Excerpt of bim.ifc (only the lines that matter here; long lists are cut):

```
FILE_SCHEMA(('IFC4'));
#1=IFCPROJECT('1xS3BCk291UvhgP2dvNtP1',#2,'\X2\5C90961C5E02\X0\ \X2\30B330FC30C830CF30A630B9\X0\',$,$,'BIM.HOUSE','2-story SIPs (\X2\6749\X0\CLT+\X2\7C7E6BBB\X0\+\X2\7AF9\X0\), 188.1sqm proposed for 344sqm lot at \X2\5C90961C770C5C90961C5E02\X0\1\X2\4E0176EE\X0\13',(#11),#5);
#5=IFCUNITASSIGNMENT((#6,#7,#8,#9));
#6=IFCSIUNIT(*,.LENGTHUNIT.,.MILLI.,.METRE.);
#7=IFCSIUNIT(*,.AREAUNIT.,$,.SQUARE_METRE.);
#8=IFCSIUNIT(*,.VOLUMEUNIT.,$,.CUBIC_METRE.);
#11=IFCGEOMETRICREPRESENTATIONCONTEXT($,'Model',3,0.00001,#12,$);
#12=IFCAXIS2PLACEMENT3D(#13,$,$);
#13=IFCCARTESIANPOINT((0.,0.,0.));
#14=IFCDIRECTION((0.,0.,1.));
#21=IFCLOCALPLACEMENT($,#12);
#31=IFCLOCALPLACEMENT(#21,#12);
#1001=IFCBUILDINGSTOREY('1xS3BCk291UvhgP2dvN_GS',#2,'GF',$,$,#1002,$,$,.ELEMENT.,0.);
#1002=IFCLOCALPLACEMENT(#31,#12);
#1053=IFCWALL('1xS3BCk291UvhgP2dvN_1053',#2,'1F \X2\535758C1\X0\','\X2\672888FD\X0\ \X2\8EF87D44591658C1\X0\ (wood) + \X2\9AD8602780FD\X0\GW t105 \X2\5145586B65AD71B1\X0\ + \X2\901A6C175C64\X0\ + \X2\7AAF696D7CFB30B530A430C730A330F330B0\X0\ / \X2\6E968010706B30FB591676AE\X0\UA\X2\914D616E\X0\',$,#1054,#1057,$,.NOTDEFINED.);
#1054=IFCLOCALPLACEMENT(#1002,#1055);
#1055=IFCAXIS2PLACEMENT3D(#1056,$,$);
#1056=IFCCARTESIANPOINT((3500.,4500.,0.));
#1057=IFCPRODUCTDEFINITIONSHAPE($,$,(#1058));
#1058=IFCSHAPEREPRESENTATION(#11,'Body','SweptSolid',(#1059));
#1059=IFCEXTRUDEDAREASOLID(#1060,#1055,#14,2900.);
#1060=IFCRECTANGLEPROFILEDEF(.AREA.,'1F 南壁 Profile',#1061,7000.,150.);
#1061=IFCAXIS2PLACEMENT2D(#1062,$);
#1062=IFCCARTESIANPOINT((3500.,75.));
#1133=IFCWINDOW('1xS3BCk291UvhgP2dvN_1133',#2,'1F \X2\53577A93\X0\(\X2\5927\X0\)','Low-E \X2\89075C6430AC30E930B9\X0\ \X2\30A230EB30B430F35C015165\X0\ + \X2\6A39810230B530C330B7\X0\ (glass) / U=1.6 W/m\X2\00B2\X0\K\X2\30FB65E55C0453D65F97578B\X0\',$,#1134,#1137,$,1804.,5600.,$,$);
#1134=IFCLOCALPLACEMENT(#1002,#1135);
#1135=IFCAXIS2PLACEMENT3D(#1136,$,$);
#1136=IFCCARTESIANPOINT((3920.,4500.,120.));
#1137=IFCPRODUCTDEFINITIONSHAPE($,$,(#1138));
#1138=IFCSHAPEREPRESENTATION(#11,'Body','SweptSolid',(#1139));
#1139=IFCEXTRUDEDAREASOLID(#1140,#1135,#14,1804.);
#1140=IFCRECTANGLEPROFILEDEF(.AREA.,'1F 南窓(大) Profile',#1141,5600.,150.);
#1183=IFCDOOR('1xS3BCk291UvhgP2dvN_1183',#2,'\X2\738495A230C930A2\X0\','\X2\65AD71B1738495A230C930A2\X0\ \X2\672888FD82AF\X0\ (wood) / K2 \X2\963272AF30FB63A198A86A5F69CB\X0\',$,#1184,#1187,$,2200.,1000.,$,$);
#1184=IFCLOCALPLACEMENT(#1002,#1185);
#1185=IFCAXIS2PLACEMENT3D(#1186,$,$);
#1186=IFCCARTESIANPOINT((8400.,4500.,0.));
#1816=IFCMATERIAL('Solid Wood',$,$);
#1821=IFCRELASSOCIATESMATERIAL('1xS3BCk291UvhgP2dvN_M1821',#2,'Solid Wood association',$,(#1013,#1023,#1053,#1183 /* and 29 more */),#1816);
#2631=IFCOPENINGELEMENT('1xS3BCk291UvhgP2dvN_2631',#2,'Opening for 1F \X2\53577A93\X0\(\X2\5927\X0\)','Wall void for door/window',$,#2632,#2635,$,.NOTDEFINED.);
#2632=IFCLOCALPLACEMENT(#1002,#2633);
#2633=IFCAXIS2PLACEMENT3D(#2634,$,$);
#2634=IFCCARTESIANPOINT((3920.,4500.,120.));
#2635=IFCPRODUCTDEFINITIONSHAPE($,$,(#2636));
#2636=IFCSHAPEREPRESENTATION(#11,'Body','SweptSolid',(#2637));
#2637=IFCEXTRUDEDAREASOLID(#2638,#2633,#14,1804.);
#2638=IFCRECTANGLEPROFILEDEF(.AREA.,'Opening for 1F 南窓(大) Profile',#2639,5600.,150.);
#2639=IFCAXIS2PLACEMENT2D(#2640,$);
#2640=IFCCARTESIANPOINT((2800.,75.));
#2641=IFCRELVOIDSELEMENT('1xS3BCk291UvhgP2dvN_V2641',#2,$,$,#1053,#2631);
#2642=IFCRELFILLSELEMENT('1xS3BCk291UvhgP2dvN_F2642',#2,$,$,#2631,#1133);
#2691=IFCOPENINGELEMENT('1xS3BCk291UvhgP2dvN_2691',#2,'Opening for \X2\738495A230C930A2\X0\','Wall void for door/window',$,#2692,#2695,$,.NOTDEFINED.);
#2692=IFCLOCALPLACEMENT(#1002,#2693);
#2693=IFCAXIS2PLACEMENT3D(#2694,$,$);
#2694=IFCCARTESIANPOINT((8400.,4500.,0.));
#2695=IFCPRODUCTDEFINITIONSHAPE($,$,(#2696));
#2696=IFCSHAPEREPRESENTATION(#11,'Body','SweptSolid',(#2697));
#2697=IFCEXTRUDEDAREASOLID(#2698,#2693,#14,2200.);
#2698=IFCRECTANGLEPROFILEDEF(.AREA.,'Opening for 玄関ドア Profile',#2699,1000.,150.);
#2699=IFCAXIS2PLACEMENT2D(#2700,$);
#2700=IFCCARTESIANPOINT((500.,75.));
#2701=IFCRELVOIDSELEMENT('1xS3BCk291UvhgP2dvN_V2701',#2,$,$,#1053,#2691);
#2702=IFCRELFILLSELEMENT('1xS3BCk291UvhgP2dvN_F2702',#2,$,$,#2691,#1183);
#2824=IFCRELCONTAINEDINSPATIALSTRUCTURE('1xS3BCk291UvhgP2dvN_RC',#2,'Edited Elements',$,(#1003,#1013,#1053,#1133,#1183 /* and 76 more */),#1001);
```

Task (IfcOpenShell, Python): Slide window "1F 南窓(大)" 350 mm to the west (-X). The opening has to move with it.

```python
import ifcopenshell
import ifcopenshell.api.geometry
import ifcopenshell.util.placement

model = ifcopenshell.open("bim.ifc")

window = model.by_guid("1xS3BCk291UvhgP2dvN_1133")
opening = window.FillsVoids[0].RelatingOpeningElement
wall = opening.VoidsElements[0].RelatingBuildingElement

wall_matrix = ifcopenshell.util.placement.get_local_placement(wall.ObjectPlacement)
shift = wall_matrix[:3, 0] * -350.0
before = ifcopenshell.util.placement.get_local_placement(window.ObjectPlacement)[:3, 3].copy()

# The window is not placed relative to its opening, so move both.
for product in (opening, window):
    matrix = ifcopenshell.util.placement.get_local_placement(product.ObjectPlacement)
    matrix[:3, 3] += shift
    ifcopenshell.api.geometry.edit_object_placement(model, product=product, matrix=matrix, is_si=False)

after = ifcopenshell.util.placement.get_local_placement(window.ObjectPlacement)[:3, 3]
print("window moved by", (after - before).round(3) + 0.0)

model.write("bim_v2.ifc")
```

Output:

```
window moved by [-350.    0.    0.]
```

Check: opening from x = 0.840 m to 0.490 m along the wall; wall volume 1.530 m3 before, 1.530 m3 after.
